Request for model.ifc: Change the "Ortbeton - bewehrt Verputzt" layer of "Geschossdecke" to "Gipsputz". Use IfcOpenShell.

First a look at what the model holds.

```python
import ifcopenshell
import ifcopenshell.util.element

model = ifcopenshell.open("model.ifc")
print(model.schema)
for layer_set in model.by_type("IfcMaterialLayerSet"):
    if layer_set.LayerSetName == "Geschossdecke":
        for layer in layer_set.MaterialLayers:
            print(layer.id(), layer.Material and layer.Material.Name, layer.LayerThickness, sep=" | ")
        print(len(ifcopenshell.util.element.get_elements_by_material(model, layer_set)), "elements and types use it")
print(sorted(m.Name for m in model.by_type("IfcMaterial") if m.Name)[:60])
```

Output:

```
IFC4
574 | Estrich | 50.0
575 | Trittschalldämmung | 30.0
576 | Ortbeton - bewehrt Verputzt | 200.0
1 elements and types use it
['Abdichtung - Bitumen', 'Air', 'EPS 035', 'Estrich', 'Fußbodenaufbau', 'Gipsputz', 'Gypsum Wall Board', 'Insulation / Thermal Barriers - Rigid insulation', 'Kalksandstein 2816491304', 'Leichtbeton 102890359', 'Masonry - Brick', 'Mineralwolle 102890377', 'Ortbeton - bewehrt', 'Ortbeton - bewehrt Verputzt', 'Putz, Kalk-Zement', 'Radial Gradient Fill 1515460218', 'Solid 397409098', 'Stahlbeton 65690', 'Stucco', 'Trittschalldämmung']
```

```python
import ifcopenshell
import ifcopenshell.api.material

model = ifcopenshell.open("model.ifc")

layer_set = next(s for s in model.by_type("IfcMaterialLayerSet") if s.LayerSetName == "Geschossdecke")
layer = next(l for l in layer_set.MaterialLayers if l.Material and l.Material.Name == "Ortbeton - bewehrt Verputzt")
material = next(m for m in model.by_type("IfcMaterial") if m.Name == "Gipsputz")

# Point this one layer at the other material; renaming the old one would change it everywhere.
ifcopenshell.api.material.edit_layer(model, layer=layer, attributes={}, material=material)

print([l.Material.Name if l.Material else None for l in layer_set.MaterialLayers])

model.write("model_rev.ifc")
```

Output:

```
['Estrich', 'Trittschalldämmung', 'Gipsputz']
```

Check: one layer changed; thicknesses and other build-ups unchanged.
